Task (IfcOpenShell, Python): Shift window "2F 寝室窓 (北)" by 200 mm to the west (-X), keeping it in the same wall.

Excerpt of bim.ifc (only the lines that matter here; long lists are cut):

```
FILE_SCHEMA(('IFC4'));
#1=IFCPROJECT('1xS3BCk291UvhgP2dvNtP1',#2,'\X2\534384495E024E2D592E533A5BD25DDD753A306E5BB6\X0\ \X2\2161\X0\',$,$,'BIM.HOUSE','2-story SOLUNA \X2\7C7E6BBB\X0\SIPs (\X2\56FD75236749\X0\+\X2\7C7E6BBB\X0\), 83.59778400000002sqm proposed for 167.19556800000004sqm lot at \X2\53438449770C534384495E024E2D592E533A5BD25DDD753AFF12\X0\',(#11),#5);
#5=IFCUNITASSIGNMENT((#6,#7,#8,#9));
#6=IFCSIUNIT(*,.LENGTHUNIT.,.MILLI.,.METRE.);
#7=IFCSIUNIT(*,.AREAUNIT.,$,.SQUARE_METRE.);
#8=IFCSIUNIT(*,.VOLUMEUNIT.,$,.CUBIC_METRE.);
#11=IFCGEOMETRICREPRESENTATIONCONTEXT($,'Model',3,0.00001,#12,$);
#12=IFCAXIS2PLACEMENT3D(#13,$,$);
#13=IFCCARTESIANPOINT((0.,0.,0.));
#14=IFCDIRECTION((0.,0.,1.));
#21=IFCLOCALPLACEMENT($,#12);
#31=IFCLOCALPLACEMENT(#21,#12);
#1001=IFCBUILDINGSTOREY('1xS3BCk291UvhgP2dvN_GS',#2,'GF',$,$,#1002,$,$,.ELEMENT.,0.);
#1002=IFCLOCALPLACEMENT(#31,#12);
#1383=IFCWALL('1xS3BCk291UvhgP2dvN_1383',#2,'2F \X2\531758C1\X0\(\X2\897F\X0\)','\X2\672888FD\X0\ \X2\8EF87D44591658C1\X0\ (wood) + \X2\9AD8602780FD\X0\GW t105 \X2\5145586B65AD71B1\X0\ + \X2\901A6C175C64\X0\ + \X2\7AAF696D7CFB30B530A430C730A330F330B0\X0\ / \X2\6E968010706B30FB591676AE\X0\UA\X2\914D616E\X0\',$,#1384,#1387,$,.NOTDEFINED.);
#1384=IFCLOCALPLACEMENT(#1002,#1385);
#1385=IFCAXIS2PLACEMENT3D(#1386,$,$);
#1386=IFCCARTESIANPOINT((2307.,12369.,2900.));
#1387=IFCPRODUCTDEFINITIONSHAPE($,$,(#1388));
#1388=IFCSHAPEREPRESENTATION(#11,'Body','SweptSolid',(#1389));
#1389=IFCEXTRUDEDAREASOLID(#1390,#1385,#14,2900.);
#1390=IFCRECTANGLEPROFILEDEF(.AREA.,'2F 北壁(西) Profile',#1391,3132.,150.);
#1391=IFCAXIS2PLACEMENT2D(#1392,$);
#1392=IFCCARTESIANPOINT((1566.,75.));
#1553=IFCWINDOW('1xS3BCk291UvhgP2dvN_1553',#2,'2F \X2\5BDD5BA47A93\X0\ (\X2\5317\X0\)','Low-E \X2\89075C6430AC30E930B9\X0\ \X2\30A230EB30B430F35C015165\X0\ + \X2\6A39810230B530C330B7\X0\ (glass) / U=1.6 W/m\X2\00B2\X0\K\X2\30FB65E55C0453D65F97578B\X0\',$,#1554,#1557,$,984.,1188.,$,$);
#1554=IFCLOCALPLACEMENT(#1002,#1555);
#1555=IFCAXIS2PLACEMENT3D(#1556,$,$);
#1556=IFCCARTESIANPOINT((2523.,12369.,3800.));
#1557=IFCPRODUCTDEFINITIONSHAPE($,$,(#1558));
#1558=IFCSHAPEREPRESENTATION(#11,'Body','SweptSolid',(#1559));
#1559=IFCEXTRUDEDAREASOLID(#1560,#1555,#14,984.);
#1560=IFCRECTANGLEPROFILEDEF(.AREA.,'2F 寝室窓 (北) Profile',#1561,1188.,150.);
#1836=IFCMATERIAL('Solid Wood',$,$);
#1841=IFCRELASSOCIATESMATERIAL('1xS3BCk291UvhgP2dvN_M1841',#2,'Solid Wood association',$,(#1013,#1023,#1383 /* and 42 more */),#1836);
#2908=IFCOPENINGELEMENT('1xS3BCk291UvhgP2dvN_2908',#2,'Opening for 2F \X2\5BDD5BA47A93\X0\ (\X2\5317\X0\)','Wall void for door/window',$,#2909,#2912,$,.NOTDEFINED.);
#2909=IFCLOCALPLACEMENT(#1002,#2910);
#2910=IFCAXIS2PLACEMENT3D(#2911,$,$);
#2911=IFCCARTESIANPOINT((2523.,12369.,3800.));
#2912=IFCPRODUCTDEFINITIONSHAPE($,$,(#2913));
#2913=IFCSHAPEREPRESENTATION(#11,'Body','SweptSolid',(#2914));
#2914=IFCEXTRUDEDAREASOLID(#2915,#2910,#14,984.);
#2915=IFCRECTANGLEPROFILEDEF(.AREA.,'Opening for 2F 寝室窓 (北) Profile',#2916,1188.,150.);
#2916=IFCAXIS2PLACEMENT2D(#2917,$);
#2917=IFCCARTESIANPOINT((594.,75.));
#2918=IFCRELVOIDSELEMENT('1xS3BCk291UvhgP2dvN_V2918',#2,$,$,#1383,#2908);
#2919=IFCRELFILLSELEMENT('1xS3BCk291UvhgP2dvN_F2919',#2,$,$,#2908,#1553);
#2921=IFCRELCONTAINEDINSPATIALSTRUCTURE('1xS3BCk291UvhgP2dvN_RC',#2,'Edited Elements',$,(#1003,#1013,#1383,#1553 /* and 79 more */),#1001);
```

```python
import ifcopenshell
import ifcopenshell.api.geometry
import ifcopenshell.util.placement

model = ifcopenshell.open("bim.ifc")

window = model.by_guid("1xS3BCk291UvhgP2dvN_1553")
opening = window.FillsVoids[0].RelatingOpeningElement
wall = opening.VoidsElements[0].RelatingBuildingElement

wall_matrix = ifcopenshell.util.placement.get_local_placement(wall.ObjectPlacement)
shift = wall_matrix[:3, 0] * -200.0
before = ifcopenshell.util.placement.get_local_placement(window.ObjectPlacement)[:3, 3].copy()

# The window is not placed relative to its opening, so move both.
for product in (opening, window):
    matrix = ifcopenshell.util.placement.get_local_placement(product.ObjectPlacement)
    matrix[:3, 3] += shift
    ifcopenshell.api.geometry.edit_object_placement(model, product=product, matrix=matrix, is_si=False)

after = ifcopenshell.util.placement.get_local_placement(window.ObjectPlacement)[:3, 3]
print("window moved by", (after - before).round(3) + 0.0)

model.write("bim_edited.ifc")
```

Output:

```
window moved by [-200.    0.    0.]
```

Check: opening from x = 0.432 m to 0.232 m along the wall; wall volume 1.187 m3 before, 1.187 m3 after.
